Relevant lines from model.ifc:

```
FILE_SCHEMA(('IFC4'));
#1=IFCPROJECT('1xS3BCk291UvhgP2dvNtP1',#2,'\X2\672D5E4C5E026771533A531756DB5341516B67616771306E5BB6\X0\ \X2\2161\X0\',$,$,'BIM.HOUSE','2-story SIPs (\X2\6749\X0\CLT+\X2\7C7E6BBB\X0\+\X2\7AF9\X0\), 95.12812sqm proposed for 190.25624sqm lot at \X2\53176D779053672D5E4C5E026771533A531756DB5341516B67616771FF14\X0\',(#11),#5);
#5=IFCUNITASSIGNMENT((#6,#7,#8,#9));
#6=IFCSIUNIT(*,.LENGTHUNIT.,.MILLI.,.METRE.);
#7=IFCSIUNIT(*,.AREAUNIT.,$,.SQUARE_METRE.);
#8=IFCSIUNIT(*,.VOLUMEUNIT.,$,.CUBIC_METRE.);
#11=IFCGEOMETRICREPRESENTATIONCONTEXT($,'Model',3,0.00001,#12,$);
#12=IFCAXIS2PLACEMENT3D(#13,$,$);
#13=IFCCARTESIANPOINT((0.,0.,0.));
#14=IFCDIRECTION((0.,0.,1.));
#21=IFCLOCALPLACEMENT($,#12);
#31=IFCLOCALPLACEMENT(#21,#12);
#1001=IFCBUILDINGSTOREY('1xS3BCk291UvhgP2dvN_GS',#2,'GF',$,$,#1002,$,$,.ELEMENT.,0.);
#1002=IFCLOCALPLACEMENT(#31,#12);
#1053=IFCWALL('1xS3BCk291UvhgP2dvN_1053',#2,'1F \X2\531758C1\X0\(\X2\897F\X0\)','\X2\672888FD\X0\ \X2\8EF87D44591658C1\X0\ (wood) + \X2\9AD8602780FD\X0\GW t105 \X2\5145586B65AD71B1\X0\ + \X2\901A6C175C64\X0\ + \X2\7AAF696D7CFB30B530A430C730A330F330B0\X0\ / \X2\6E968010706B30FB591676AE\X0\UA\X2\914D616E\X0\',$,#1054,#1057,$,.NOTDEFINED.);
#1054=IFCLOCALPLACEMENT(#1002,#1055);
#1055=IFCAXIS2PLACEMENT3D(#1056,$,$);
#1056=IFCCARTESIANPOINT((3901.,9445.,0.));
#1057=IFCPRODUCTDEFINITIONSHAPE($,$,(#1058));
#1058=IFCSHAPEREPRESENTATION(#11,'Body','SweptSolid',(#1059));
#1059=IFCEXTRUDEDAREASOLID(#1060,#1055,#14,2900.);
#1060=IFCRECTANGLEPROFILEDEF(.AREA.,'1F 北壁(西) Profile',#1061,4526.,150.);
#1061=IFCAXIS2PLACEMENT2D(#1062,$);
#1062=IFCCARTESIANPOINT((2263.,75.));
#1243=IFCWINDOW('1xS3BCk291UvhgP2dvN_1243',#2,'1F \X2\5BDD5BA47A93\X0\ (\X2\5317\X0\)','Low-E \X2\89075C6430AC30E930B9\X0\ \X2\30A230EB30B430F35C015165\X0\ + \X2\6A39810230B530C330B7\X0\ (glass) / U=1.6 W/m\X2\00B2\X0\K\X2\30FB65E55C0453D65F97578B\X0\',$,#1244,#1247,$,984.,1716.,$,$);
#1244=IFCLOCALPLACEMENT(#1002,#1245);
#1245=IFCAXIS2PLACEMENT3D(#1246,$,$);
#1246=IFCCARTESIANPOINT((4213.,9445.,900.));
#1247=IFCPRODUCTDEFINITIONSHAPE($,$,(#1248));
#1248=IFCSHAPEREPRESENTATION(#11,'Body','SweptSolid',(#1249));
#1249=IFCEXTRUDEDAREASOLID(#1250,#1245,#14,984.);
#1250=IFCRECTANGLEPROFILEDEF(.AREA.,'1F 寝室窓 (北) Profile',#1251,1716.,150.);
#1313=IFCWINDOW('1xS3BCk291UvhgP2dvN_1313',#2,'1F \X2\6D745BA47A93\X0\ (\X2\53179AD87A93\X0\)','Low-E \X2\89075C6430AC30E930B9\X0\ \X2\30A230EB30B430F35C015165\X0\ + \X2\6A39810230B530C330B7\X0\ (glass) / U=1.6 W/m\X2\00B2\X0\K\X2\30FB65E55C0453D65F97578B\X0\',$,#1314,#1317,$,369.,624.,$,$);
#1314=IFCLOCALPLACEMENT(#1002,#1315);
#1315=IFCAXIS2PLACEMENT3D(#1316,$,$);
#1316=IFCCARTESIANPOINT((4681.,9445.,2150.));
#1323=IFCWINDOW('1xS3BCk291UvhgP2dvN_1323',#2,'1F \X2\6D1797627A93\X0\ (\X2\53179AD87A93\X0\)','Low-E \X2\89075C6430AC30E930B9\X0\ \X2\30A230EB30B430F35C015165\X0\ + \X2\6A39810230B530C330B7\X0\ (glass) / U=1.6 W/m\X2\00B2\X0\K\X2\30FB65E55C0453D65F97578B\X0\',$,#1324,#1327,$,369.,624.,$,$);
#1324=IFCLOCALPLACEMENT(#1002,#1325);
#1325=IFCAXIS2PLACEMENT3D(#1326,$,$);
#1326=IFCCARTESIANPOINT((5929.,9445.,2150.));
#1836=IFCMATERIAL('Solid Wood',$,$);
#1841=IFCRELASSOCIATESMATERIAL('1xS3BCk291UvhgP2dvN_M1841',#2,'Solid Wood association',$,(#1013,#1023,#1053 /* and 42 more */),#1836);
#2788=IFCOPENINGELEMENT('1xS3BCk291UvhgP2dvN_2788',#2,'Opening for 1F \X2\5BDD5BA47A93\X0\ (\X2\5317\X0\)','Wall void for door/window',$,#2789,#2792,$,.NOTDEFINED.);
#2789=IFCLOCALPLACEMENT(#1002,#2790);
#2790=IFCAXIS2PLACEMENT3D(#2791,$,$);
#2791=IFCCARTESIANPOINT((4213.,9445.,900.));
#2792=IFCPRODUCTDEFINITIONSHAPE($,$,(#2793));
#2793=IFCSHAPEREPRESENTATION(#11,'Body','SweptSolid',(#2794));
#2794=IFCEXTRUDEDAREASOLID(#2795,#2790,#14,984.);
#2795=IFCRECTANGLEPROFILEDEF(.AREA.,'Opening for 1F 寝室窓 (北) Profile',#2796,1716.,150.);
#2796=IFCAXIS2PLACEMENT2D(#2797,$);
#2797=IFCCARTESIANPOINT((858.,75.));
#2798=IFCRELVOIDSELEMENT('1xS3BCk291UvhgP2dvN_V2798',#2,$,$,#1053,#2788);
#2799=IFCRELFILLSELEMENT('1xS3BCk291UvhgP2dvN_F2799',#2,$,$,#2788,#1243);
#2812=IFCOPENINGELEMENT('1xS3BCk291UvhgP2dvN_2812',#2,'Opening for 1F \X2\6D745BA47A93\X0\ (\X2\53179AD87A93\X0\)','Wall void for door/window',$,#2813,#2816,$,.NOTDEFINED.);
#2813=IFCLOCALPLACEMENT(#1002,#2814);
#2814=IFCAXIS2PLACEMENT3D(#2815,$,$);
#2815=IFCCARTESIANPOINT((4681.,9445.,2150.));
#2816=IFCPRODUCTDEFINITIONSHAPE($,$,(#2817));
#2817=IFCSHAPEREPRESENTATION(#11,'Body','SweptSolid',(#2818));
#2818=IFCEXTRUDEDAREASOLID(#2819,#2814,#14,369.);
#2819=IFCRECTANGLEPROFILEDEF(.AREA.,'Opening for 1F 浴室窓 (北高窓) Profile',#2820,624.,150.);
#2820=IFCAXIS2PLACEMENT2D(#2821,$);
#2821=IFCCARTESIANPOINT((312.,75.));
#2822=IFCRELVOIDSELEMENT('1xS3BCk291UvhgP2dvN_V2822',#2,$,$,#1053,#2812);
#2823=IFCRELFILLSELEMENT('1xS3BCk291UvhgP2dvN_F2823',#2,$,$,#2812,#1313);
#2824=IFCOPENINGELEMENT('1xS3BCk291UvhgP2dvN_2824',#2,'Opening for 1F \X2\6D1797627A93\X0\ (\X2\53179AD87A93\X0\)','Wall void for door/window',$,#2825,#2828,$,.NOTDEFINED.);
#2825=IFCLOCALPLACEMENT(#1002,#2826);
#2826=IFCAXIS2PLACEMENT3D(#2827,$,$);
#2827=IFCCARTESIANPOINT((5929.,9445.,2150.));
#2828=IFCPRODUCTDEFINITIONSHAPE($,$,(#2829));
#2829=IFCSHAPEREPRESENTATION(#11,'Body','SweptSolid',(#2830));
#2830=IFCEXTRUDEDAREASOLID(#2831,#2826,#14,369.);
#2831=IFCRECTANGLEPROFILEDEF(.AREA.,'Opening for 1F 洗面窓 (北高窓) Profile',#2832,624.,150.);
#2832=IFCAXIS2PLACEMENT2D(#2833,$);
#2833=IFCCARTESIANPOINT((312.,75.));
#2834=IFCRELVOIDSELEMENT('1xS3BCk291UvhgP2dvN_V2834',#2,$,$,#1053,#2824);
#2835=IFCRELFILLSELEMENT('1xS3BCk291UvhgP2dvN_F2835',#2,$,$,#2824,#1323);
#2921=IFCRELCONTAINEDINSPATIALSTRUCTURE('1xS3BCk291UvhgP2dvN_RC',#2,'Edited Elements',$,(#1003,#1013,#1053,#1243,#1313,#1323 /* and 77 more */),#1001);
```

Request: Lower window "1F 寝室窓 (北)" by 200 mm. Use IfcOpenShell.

```python
import numpy as np
import ifcopenshell
import ifcopenshell.api.geometry
import ifcopenshell.util.placement
import ifcopenshell.util.unit

model = ifcopenshell.open("model.ifc")
unit_scale = ifcopenshell.util.unit.calculate_unit_scale(model)

window = model.by_guid("1xS3BCk291UvhgP2dvN_1243")
opening = window.FillsVoids[0].RelatingOpeningElement
dz = -0.2 / unit_scale

shift = np.array([0.0, 0.0, dz])
# The window is not placed relative to its opening, so move both.
for product in (opening, window):
    matrix = ifcopenshell.util.placement.get_local_placement(product.ObjectPlacement)
    matrix[:3, 3] += shift
    ifcopenshell.api.geometry.edit_object_placement(model, product=product, matrix=matrix, is_si=False)

print(f"moved by {dz * unit_scale:+.3f} m")

model.write("model_updated.ifc")
```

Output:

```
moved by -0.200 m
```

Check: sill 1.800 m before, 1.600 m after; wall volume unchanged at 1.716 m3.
